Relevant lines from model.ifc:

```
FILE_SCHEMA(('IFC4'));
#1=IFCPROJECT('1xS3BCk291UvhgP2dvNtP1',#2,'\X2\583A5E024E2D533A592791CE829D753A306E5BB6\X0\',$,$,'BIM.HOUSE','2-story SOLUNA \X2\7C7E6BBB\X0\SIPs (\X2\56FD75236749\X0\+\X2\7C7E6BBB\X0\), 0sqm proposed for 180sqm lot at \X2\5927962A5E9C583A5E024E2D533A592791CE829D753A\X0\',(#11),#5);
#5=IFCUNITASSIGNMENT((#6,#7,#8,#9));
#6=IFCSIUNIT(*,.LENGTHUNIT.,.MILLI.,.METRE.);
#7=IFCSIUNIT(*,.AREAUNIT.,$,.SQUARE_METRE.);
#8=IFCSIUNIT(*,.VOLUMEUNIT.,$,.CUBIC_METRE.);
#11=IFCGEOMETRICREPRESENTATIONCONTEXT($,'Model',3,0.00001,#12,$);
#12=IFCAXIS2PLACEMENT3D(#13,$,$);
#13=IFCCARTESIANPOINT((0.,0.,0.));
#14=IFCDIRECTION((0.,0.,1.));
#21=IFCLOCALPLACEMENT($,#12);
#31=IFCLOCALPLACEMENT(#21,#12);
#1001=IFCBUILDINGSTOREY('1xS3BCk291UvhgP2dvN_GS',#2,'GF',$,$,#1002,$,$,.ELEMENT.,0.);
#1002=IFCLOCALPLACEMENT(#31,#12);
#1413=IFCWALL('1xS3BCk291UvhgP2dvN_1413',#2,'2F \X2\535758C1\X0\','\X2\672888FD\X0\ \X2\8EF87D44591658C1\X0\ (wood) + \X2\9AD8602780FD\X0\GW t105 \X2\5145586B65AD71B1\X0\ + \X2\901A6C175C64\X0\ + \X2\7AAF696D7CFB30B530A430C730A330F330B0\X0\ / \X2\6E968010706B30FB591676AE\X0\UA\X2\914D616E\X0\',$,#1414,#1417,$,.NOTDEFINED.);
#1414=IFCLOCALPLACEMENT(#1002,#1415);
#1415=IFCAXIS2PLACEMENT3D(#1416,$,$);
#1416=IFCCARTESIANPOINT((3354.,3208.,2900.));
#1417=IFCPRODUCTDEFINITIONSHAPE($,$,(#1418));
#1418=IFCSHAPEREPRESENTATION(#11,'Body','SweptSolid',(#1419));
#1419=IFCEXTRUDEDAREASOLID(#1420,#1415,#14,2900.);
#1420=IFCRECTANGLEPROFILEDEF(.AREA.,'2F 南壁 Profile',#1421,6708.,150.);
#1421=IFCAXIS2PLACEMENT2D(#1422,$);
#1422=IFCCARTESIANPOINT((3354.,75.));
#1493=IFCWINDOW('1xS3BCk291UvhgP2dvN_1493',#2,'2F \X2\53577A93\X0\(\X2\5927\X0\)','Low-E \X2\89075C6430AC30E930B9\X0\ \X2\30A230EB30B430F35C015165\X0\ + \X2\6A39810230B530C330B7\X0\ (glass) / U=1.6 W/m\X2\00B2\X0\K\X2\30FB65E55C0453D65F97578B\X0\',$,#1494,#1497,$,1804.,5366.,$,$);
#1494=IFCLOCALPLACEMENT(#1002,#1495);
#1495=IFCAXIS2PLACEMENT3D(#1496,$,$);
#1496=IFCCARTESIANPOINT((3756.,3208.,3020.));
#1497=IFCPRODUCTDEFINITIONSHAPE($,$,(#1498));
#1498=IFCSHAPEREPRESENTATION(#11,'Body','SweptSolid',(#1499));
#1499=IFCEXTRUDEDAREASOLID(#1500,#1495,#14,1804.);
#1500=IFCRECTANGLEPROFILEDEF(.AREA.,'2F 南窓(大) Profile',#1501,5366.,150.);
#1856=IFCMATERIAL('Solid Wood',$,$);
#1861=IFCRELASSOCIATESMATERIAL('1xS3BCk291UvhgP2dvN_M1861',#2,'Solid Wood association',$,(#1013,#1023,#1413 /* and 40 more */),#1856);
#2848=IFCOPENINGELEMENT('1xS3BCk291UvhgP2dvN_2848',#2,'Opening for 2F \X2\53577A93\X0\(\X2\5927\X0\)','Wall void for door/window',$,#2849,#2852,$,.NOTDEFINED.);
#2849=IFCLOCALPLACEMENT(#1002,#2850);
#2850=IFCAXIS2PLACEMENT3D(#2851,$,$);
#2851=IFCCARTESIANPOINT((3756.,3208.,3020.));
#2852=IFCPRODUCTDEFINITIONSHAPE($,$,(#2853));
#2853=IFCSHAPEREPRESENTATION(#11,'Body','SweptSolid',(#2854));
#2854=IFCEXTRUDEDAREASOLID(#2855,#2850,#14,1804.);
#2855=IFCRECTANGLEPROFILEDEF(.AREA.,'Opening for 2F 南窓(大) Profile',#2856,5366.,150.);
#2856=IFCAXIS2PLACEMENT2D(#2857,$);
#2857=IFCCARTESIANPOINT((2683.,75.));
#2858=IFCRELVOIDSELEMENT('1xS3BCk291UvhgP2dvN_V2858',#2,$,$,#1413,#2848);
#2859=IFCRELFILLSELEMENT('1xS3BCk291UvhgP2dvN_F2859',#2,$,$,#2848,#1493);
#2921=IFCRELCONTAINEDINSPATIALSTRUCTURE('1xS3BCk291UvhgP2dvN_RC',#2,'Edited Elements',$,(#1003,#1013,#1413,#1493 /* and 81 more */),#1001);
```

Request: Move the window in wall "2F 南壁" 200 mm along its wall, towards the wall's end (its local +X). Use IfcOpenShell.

```python
import ifcopenshell
import ifcopenshell.api.geometry
import ifcopenshell.util.placement
import ifcopenshell.util.unit

model = ifcopenshell.open("model.ifc")
unit_scale = ifcopenshell.util.unit.calculate_unit_scale(model)

window = model.by_guid("1xS3BCk291UvhgP2dvN_1493")
opening = window.FillsVoids[0].RelatingOpeningElement
wall = opening.VoidsElements[0].RelatingBuildingElement

wall_matrix = ifcopenshell.util.placement.get_local_placement(wall.ObjectPlacement)
shift = wall_matrix[:3, 0] * 0.2 / unit_scale
before = ifcopenshell.util.placement.get_local_placement(window.ObjectPlacement)[:3, 3].copy()

# The window is not placed relative to its opening, so move both.
for product in (opening, window):
    matrix = ifcopenshell.util.placement.get_local_placement(product.ObjectPlacement)
    matrix[:3, 3] += shift
    ifcopenshell.api.geometry.edit_object_placement(model, product=product, matrix=matrix, is_si=False)

after = ifcopenshell.util.placement.get_local_placement(window.ObjectPlacement)[:3, 3]
print("window moved by", (after - before).round(3) + 0.0)

model.write("model_v2.ifc")
```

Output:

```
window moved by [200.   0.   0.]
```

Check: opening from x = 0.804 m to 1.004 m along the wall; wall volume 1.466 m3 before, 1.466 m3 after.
